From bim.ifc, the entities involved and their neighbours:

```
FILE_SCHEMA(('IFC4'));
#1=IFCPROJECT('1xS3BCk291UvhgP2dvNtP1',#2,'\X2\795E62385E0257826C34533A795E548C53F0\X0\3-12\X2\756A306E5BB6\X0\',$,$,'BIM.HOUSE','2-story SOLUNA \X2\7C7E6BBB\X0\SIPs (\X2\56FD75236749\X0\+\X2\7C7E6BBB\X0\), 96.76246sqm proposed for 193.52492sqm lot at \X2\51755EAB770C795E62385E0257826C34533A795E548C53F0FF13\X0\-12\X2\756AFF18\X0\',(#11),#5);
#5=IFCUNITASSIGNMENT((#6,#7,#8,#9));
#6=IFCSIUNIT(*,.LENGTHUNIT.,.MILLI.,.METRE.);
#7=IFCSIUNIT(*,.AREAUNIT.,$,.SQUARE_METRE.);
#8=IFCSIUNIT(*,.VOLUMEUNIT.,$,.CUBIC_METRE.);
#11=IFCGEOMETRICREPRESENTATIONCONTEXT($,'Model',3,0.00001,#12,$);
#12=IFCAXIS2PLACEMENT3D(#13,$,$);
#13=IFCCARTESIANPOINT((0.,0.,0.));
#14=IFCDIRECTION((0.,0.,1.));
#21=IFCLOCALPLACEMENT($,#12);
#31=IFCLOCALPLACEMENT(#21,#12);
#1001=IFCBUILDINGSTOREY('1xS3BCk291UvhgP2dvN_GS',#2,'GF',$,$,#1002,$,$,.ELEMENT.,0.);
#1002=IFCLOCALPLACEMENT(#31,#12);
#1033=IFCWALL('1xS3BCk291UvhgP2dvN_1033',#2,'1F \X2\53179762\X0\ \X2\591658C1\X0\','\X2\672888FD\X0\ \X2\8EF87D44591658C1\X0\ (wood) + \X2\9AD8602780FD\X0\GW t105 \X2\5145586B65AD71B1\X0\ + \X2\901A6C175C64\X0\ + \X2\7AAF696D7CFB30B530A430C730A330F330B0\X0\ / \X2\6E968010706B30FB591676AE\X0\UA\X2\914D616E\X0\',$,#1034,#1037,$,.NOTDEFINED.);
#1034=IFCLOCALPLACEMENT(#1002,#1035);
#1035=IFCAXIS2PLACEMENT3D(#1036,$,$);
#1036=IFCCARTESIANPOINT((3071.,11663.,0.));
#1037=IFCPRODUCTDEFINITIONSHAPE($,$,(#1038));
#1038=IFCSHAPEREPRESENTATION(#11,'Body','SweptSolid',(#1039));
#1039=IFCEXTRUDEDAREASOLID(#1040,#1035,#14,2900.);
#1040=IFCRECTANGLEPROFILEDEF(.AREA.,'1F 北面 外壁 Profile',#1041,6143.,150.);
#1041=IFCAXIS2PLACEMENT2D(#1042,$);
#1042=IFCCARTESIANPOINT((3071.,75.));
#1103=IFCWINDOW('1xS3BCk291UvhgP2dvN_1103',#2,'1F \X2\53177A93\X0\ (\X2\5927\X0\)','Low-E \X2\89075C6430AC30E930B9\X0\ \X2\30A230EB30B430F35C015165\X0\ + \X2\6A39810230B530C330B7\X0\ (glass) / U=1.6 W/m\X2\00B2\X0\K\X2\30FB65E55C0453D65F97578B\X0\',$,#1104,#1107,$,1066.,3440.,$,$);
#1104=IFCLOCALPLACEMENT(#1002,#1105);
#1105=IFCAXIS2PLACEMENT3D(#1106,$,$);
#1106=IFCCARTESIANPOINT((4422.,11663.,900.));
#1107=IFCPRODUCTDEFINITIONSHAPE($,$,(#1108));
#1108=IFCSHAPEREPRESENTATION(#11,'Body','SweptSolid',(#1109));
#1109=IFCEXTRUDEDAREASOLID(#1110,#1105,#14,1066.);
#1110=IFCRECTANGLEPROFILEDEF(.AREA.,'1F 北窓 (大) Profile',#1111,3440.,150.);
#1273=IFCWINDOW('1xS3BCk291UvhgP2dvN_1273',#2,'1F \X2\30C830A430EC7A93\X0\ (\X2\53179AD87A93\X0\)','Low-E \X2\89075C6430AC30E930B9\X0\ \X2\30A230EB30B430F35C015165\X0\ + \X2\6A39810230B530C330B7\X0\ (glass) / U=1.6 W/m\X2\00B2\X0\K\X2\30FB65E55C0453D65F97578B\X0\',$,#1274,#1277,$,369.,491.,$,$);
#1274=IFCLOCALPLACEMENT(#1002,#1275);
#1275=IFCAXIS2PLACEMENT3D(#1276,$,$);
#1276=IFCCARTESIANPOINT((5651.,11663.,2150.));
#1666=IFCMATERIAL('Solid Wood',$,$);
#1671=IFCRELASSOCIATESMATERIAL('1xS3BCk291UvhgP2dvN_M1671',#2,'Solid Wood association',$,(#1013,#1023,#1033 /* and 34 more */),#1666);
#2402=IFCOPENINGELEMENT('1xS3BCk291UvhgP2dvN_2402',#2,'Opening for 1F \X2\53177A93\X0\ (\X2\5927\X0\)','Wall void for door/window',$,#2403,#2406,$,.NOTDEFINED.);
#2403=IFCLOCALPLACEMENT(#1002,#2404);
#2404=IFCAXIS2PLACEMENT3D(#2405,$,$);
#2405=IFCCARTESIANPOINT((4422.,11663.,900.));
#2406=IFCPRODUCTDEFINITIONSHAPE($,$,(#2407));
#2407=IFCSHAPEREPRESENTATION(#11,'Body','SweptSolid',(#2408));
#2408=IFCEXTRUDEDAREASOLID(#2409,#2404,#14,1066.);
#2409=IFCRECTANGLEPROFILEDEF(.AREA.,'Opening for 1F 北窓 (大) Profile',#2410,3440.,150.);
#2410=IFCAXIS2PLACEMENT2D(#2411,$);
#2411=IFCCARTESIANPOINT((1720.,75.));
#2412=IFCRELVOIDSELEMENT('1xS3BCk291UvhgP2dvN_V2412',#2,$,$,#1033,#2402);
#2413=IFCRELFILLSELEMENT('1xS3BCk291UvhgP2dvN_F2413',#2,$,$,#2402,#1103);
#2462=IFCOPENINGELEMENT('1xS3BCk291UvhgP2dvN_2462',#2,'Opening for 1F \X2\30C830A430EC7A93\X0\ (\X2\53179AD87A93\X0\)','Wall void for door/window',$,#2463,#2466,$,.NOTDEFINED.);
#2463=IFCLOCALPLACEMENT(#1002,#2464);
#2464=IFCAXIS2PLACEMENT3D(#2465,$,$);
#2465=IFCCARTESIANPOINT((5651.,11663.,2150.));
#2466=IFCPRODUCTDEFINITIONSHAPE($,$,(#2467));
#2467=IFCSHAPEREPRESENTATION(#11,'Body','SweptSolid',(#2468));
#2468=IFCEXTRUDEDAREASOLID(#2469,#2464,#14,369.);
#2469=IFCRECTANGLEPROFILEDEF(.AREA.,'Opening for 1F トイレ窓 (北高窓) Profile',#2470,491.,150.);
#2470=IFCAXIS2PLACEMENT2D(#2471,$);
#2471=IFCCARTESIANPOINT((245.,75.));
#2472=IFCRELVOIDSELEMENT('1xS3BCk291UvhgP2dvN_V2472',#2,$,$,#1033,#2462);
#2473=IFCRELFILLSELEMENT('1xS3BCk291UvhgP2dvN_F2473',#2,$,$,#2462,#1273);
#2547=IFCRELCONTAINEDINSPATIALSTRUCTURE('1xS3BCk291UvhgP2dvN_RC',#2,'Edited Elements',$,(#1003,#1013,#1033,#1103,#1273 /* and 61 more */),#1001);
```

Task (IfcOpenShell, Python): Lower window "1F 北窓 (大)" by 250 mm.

```python
import numpy as np
import ifcopenshell
import ifcopenshell.api.geometry
import ifcopenshell.util.placement
import ifcopenshell.util.unit

model = ifcopenshell.open("bim.ifc")
unit_scale = ifcopenshell.util.unit.calculate_unit_scale(model)

window = model.by_guid("1xS3BCk291UvhgP2dvN_1103")
opening = window.FillsVoids[0].RelatingOpeningElement
dz = -0.25 / unit_scale

shift = np.array([0.0, 0.0, dz])
# The window is not placed relative to its opening, so move both.
for product in (opening, window):
    matrix = ifcopenshell.util.placement.get_local_placement(product.ObjectPlacement)
    matrix[:3, 3] += shift
    ifcopenshell.api.geometry.edit_object_placement(model, product=product, matrix=matrix, is_si=False)

print(f"moved by {dz * unit_scale:+.3f} m")

model.write("bim-out.ifc")
```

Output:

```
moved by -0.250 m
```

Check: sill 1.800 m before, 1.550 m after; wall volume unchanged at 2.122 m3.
